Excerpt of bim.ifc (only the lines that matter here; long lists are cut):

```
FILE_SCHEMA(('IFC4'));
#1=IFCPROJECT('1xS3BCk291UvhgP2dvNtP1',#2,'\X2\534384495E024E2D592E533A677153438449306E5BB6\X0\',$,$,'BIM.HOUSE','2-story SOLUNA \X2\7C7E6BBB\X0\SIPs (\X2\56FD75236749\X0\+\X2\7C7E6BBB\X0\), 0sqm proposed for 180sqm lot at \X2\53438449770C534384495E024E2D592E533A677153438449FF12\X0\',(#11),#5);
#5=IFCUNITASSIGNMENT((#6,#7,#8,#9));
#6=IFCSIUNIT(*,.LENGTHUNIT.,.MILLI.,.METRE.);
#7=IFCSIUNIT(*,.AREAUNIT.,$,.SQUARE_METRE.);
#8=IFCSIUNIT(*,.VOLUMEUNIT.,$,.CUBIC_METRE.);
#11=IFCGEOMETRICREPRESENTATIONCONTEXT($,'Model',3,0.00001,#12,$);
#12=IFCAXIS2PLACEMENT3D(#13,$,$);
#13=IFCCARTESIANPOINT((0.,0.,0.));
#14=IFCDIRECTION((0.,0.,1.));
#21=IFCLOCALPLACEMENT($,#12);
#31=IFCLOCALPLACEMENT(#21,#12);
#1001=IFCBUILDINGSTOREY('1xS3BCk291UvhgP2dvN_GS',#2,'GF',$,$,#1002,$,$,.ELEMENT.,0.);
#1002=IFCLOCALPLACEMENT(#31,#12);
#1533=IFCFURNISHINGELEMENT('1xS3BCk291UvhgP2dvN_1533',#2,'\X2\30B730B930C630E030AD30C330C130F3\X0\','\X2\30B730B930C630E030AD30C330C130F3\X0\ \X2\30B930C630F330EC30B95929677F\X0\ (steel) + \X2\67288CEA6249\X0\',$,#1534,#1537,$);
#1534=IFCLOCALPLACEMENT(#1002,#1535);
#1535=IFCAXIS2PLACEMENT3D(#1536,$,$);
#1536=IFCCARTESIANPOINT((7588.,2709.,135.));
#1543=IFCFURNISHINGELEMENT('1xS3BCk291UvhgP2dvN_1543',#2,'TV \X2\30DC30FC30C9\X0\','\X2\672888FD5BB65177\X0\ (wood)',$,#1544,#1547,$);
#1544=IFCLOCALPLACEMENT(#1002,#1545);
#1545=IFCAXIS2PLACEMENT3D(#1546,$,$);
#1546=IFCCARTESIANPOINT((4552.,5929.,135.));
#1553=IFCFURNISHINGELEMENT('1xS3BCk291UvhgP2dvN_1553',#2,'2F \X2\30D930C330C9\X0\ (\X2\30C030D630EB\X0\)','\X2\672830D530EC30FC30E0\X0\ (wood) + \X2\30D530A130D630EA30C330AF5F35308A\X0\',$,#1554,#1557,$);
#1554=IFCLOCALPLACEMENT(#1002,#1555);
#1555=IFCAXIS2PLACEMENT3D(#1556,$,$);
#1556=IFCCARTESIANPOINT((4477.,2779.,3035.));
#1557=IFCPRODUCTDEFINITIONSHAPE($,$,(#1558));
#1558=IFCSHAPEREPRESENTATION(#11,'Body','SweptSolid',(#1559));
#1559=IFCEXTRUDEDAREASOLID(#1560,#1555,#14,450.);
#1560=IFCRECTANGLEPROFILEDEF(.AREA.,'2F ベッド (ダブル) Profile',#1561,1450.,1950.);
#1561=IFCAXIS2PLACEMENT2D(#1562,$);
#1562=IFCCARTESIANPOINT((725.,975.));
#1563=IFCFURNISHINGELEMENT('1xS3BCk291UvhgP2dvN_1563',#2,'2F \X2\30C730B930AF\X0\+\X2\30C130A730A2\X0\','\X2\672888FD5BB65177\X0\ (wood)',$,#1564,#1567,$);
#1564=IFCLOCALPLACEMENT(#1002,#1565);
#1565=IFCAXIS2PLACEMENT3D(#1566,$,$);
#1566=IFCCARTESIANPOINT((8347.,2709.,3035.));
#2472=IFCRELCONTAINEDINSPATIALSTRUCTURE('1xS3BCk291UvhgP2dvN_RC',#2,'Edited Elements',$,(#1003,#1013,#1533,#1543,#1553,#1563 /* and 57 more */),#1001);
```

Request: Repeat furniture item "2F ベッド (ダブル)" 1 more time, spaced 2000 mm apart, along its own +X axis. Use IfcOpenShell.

```python
import ifcopenshell
import ifcopenshell.api.geometry
import ifcopenshell.api.root
import ifcopenshell.util.element
import ifcopenshell.util.placement

model = ifcopenshell.open("bim.ifc")


def reuse_history(source, copy):
    """copy_class also copies each property set's owner history, people and application; keep the originals."""
    for rel in copy.IsDefinedBy:
        if rel.is_a("IfcRelDefinesByProperties") and (history := rel.RelatingPropertyDefinition.OwnerHistory):
            rel.RelatingPropertyDefinition.OwnerHistory = source.OwnerHistory
            ifcopenshell.util.element.remove_deep2(model, history)


source = model.by_guid("1xS3BCk291UvhgP2dvN_1553")
base = ifcopenshell.util.placement.get_local_placement(source.ObjectPlacement)
step = base[:3, 0] * 2000.0

for i in range(1, 2):
    copy = ifcopenshell.api.root.copy_class(model, product=source)
    copy.Representation = ifcopenshell.util.element.copy_deep(
        model, source.Representation, exclude=["IfcGeometricRepresentationContext", "IfcRepresentationMap"]
    )
    reuse_history(source, copy)
    matrix = base.copy()
    matrix[:3, 3] += i * step
    print("added at", matrix[:3, 3].round(3) + 0.0)
    ifcopenshell.api.geometry.edit_object_placement(model, product=copy, matrix=matrix, is_si=False)

model.write("bim_v2.ifc")
```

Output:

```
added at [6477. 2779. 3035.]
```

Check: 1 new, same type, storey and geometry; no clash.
